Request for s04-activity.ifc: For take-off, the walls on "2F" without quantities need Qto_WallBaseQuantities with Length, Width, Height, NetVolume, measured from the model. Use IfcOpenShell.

First a look at what the model holds.

```python
import ifcopenshell
import ifcopenshell.util.element
import ifcopenshell.util.unit

model = ifcopenshell.open("s04-activity.ifc")
print(model.schema)
for unit_type in ("LENGTHUNIT", "AREAUNIT", "VOLUMEUNIT"):
    print(unit_type, ifcopenshell.util.unit.calculate_unit_scale(model, unit_type))
storey = next(s for s in model.by_type("IfcBuildingStorey") if s.Name == "2F")
walls = [e for e in ifcopenshell.util.element.get_decomposition(storey) if e.is_a("IfcWall")]
for e in sorted(walls, key=lambda e: e.id()):
    print(e.id(), e.is_a(), e.Name, list(ifcopenshell.util.element.get_psets(e, qtos_only=True)), sep=" | ")
```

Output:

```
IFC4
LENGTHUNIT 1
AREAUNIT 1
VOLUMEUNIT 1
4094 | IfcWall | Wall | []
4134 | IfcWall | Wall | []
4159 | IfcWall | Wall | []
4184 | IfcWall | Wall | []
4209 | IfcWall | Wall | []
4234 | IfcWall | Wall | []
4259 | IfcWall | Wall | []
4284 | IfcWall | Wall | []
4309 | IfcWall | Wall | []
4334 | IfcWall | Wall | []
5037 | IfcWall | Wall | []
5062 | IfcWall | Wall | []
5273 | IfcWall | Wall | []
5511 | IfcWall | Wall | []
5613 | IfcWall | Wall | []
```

```python
import ifcopenshell
import ifcopenshell.api.pset
import ifcopenshell.geom
import ifcopenshell.util.element
import ifcopenshell.util.shape
import ifcopenshell.util.unit

model = ifcopenshell.open("s04-activity.ifc")
unit_scale = ifcopenshell.util.unit.calculate_unit_scale(model)
volume_scale = ifcopenshell.util.unit.calculate_unit_scale(model, "VOLUMEUNIT")
settings = ifcopenshell.geom.settings()

storey = next(s for s in model.by_type("IfcBuildingStorey") if s.Name == "2F")
walls = [e for e in ifcopenshell.util.element.get_decomposition(storey) if e.is_a("IfcWall")]

for e in sorted(walls, key=lambda e: e.id()):
    if ifcopenshell.util.element.get_psets(e, qtos_only=True, should_inherit=False):
        continue
    # Geometry comes back in metres, in the element's own axes.
    shape = ifcopenshell.geom.create_shape(settings, e)
    values = {
        "Length": ifcopenshell.util.shape.get_x(shape.geometry) / unit_scale,
        "Width": ifcopenshell.util.shape.get_y(shape.geometry) / unit_scale,
        "Height": ifcopenshell.util.shape.get_z(shape.geometry) / unit_scale,
        "NetVolume": ifcopenshell.util.shape.get_volume(shape.geometry) / volume_scale,
    }
    qto = ifcopenshell.api.pset.add_qto(model, product=e, name="Qto_WallBaseQuantities")
    ifcopenshell.api.pset.edit_qto(model, qto=qto, properties=values)
    print(e.id(), {k: round(v, 3) for k, v in values.items()})

model.write("s04-activity_rev.ifc")
```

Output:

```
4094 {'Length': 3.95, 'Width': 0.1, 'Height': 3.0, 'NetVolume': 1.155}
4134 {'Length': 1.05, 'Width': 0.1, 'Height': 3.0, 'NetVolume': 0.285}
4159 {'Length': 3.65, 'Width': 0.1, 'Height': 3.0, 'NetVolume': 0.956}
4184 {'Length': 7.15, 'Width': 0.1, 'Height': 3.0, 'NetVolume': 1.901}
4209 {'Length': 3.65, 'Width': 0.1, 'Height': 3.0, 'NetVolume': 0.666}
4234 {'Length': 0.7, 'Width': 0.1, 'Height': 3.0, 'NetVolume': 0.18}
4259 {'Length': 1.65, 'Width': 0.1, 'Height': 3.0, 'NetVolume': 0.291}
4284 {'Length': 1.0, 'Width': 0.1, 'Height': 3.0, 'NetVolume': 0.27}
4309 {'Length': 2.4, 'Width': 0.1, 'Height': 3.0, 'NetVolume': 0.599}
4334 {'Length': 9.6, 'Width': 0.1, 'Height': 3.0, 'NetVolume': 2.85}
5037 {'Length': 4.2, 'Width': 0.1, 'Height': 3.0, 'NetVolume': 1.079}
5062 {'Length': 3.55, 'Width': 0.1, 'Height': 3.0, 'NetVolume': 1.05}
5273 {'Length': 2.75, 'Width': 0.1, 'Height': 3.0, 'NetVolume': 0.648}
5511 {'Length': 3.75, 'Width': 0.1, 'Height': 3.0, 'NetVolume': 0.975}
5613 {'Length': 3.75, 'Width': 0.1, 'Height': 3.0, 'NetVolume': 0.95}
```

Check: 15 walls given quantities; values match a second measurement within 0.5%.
